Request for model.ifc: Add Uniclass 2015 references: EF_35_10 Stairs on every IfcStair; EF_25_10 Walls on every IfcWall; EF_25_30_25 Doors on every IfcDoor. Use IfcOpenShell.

First a look at what the model holds.

```python
import ifcopenshell

model = ifcopenshell.open("model.ifc")
print(model.schema)
print("classifications:", [c.Name for c in model.by_type("IfcClassification")])
for ifc_class in ("IfcDoor", "IfcRoof", "IfcStair", "IfcWall", "IfcWindow"):
    print(ifc_class, len(model.by_type(ifc_class)))
```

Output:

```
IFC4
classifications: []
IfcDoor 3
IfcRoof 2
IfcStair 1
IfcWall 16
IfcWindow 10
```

```python
import ifcopenshell
import ifcopenshell.api.classification

model = ifcopenshell.open("model.ifc")

system = ifcopenshell.api.classification.add_classification(model, classification="Uniclass 2015")

codes = {
    "IfcStair": ("EF_35_10", "Stairs"),
    "IfcWall": ("EF_25_10", "Walls"),
    "IfcDoor": ("EF_25_30_25", "Doors"),
}
for ifc_class, (code, name) in codes.items():
    products = model.by_type(ifc_class)
    ifcopenshell.api.classification.add_reference(
        model, products=products, classification=system, identification=code, name=name
    )
    print(code, len(products))

model.write("model_updated.ifc")
```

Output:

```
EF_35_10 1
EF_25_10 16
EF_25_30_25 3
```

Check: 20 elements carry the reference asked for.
